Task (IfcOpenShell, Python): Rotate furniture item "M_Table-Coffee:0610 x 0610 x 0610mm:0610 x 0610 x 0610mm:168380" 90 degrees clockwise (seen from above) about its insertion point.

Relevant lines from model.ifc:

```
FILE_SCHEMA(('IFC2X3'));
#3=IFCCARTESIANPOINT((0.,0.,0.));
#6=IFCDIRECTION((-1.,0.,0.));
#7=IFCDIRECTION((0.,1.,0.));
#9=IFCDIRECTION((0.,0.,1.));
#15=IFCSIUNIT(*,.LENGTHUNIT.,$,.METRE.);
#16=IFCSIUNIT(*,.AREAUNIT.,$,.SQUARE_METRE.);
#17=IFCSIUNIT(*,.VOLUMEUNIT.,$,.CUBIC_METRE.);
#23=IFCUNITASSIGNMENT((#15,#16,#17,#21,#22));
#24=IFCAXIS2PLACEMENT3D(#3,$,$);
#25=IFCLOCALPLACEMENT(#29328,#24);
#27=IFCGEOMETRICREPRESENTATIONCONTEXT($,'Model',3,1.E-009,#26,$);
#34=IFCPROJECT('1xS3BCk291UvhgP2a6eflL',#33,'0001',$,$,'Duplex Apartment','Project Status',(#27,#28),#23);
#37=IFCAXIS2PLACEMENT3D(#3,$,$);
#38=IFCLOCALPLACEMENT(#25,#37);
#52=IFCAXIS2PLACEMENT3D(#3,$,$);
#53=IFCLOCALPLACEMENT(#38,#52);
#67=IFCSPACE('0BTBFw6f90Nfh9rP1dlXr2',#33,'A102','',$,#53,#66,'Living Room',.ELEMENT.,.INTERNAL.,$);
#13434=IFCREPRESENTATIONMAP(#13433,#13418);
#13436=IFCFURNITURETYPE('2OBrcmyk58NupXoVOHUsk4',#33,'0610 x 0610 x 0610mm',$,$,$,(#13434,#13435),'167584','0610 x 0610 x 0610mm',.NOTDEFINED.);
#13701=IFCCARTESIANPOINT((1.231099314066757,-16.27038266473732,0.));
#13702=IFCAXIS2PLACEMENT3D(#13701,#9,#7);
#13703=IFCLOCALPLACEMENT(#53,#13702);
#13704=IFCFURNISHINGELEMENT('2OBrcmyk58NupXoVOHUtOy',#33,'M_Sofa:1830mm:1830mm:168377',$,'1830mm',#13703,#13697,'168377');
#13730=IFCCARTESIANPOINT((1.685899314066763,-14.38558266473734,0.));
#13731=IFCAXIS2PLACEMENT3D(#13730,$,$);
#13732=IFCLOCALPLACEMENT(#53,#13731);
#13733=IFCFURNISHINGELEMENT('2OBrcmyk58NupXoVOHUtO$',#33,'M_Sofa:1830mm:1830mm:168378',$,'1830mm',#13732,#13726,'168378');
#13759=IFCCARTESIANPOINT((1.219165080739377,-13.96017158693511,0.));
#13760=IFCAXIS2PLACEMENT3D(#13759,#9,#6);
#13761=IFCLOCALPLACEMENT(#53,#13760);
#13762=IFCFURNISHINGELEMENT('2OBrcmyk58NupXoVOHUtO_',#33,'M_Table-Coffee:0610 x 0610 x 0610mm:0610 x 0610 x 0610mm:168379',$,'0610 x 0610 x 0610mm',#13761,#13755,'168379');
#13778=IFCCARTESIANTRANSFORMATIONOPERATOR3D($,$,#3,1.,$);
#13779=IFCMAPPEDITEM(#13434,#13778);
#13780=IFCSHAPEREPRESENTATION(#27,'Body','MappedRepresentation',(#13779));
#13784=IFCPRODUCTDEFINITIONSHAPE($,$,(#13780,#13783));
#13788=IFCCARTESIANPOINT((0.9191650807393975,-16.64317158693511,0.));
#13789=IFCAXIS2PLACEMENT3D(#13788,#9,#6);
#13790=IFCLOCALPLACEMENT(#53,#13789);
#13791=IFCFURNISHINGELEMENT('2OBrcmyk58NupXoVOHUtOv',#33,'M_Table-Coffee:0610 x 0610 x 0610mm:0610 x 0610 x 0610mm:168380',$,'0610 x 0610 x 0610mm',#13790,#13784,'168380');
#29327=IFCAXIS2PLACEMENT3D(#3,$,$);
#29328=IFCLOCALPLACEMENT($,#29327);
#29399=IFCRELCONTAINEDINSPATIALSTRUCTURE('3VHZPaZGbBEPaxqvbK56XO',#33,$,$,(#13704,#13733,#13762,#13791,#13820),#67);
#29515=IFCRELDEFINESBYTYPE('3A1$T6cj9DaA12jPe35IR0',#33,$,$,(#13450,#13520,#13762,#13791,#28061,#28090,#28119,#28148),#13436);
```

```python
import ifcopenshell
import ifcopenshell.api.geometry
import ifcopenshell.util.placement

model = ifcopenshell.open("model.ifc")

item = model.by_guid("2OBrcmyk58NupXoVOHUtOv")
matrix = ifcopenshell.util.placement.get_local_placement(item.ObjectPlacement)
matrix = matrix @ ifcopenshell.util.placement.rotation(-90, "Z")
ifcopenshell.api.geometry.edit_object_placement(model, product=item, matrix=matrix, is_si=False)

print(ifcopenshell.util.placement.get_local_placement(item.ObjectPlacement).round(3) + 0.0)

model.write("model_updated.ifc")
```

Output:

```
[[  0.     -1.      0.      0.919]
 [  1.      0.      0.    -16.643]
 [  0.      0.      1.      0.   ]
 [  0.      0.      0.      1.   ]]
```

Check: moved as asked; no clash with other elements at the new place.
